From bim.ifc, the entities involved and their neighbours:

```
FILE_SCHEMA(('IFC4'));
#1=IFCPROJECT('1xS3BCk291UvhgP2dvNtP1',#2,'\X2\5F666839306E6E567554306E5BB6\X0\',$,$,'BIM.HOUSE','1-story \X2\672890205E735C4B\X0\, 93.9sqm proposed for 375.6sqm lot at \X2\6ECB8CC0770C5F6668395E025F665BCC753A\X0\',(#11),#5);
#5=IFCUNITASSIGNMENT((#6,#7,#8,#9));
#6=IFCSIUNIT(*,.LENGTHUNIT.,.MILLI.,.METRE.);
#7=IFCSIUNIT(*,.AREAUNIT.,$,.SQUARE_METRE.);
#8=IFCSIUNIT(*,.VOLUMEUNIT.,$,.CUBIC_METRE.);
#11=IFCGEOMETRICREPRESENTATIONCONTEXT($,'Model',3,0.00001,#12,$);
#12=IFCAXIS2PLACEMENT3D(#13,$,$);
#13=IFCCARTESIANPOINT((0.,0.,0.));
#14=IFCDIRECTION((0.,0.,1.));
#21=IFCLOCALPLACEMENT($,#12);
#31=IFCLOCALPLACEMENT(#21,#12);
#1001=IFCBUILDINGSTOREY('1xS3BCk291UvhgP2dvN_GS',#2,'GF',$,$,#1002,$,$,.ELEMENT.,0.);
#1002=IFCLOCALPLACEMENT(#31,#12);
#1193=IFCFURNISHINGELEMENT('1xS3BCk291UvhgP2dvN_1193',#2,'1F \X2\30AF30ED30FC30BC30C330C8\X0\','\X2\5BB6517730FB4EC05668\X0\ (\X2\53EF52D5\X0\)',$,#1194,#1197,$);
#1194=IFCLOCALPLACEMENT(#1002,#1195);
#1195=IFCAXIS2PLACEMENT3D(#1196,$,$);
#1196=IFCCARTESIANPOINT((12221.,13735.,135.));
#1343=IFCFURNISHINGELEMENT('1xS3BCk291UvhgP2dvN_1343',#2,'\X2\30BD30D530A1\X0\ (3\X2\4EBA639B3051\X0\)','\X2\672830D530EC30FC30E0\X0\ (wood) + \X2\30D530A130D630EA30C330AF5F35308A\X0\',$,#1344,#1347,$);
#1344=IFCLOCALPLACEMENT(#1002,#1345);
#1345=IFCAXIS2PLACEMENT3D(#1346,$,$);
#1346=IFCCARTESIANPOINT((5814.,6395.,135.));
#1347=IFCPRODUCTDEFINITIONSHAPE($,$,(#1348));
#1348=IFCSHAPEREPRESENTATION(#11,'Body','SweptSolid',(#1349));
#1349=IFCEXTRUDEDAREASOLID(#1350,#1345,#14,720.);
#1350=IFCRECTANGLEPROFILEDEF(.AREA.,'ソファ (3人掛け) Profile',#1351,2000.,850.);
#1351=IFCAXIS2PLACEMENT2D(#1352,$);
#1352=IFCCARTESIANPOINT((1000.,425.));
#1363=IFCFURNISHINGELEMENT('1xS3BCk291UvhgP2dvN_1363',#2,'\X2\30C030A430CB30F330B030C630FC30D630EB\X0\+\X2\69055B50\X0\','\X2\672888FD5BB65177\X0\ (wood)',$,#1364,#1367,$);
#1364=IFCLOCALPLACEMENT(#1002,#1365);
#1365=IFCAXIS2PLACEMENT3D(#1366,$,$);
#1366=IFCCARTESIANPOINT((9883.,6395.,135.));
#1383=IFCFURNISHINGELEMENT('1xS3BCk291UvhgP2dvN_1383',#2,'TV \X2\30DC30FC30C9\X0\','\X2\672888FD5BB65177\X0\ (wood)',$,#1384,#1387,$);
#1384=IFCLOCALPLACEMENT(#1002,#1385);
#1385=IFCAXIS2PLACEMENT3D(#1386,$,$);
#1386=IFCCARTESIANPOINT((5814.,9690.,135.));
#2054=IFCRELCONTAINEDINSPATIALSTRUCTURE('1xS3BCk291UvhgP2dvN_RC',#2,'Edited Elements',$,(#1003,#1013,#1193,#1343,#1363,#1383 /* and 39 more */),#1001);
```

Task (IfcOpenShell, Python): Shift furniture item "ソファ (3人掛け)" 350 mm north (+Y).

```python
import ifcopenshell
import ifcopenshell.api.geometry
import ifcopenshell.util.placement

model = ifcopenshell.open("bim.ifc")

item = model.by_guid("1xS3BCk291UvhgP2dvN_1343")
matrix = ifcopenshell.util.placement.get_local_placement(item.ObjectPlacement)
matrix[1, 3] += 350.0
ifcopenshell.api.geometry.edit_object_placement(model, product=item, matrix=matrix, is_si=False)

print(ifcopenshell.util.placement.get_local_placement(item.ObjectPlacement).round(3) + 0.0)

model.write("bim_updated.ifc")
```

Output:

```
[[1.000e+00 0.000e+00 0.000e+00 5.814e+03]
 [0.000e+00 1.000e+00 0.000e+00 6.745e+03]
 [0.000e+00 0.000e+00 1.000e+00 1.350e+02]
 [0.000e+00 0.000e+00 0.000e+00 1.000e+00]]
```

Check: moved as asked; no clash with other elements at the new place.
